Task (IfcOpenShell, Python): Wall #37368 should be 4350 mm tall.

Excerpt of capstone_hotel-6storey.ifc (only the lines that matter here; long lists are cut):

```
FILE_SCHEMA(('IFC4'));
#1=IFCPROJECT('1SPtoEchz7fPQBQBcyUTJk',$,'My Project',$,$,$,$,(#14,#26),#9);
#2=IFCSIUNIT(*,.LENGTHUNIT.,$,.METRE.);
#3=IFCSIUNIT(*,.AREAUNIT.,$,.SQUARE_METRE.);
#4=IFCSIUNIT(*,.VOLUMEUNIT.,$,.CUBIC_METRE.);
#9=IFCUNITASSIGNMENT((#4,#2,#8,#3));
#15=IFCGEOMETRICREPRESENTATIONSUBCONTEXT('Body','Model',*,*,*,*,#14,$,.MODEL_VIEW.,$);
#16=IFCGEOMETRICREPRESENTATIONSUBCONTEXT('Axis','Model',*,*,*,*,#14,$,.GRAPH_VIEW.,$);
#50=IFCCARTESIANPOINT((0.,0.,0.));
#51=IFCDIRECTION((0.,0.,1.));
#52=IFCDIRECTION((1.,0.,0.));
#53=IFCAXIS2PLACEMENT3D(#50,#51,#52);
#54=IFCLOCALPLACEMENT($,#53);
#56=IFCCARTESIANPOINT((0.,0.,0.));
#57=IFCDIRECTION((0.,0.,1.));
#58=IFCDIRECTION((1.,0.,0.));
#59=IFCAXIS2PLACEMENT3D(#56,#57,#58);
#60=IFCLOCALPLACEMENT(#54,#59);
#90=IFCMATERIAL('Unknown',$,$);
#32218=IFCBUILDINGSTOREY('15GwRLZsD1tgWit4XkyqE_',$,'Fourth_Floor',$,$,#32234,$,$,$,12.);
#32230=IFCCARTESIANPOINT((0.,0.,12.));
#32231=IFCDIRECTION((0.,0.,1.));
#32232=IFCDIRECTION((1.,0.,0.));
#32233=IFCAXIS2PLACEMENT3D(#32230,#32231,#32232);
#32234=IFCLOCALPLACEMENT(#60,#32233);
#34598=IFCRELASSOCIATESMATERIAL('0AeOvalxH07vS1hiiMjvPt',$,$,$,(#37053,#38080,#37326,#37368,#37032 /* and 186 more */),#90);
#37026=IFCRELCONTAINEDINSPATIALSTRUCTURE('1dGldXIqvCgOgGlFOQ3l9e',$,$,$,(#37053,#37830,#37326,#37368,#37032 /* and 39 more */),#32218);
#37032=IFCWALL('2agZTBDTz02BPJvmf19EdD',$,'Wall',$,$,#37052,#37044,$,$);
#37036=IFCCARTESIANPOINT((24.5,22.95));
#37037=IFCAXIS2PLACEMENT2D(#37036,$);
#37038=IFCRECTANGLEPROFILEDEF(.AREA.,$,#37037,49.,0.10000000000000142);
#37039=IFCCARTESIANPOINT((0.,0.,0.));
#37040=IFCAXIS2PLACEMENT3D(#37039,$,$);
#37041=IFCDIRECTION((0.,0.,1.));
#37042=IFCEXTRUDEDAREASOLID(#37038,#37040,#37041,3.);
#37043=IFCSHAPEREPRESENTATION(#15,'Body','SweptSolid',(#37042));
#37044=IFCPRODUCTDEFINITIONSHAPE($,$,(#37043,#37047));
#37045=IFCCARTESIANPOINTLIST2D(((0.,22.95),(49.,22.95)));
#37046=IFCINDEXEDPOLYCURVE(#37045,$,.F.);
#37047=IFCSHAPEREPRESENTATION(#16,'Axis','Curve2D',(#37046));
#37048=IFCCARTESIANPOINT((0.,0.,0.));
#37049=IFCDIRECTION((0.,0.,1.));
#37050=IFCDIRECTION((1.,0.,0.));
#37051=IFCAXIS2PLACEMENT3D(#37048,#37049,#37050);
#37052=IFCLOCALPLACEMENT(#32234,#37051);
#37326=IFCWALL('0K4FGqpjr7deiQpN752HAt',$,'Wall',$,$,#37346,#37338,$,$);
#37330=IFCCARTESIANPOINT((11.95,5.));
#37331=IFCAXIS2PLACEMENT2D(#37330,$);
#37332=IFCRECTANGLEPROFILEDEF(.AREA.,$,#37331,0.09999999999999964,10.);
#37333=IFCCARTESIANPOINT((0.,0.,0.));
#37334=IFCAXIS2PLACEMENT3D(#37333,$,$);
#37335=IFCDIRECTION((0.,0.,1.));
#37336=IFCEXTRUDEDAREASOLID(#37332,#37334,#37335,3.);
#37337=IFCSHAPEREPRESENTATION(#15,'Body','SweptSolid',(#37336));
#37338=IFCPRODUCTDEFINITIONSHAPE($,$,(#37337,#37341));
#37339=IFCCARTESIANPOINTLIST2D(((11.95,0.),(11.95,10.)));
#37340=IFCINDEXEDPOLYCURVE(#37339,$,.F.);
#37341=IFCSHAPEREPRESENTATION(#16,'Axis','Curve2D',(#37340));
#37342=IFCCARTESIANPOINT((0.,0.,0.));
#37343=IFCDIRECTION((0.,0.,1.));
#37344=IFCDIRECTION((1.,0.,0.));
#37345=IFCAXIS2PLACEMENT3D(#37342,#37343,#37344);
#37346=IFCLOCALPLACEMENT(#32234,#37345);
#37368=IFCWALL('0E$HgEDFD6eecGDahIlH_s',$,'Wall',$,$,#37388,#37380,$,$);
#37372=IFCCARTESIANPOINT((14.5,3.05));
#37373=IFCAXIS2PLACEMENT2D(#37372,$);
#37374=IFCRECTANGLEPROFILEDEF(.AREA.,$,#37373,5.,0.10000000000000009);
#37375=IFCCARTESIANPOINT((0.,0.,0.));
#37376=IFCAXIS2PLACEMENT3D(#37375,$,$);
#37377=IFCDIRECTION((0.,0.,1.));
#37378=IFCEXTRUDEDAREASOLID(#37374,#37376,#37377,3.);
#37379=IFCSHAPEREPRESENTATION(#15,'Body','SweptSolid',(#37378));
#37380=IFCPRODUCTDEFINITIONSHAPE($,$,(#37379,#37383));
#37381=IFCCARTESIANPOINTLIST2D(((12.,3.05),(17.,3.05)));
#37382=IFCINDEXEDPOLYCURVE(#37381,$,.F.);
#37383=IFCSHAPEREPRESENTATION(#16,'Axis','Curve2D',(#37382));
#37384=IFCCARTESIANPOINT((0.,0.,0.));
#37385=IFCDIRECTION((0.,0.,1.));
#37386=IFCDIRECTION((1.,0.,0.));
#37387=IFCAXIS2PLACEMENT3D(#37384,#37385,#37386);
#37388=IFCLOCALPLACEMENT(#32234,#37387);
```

```python
import ifcopenshell
import ifcopenshell.geom
import ifcopenshell.util.representation
import ifcopenshell.util.shape

model = ifcopenshell.open("capstone_hotel-6storey.ifc")
settings = ifcopenshell.geom.settings()


def volume(element):
    """Net volume in cubic metres, openings subtracted."""
    shape = ifcopenshell.geom.create_shape(settings, element)
    return ifcopenshell.util.shape.get_volume(shape.geometry)


wall = model.by_id(37368)
before = volume(wall)

body = ifcopenshell.util.representation.get_representation(wall, "Model", "Body")
solid = body.Items[0]
old_height = solid.Depth
solid.Depth = 4.35
after = volume(wall)

print(f"height {old_height:g} -> {solid.Depth:g}, volume {before:.3f} -> {after:.3f} m3")

model.write("capstone_hotel-6storey_v2.ifc")
```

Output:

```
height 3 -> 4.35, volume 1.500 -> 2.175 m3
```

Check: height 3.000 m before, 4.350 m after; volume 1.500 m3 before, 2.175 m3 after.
